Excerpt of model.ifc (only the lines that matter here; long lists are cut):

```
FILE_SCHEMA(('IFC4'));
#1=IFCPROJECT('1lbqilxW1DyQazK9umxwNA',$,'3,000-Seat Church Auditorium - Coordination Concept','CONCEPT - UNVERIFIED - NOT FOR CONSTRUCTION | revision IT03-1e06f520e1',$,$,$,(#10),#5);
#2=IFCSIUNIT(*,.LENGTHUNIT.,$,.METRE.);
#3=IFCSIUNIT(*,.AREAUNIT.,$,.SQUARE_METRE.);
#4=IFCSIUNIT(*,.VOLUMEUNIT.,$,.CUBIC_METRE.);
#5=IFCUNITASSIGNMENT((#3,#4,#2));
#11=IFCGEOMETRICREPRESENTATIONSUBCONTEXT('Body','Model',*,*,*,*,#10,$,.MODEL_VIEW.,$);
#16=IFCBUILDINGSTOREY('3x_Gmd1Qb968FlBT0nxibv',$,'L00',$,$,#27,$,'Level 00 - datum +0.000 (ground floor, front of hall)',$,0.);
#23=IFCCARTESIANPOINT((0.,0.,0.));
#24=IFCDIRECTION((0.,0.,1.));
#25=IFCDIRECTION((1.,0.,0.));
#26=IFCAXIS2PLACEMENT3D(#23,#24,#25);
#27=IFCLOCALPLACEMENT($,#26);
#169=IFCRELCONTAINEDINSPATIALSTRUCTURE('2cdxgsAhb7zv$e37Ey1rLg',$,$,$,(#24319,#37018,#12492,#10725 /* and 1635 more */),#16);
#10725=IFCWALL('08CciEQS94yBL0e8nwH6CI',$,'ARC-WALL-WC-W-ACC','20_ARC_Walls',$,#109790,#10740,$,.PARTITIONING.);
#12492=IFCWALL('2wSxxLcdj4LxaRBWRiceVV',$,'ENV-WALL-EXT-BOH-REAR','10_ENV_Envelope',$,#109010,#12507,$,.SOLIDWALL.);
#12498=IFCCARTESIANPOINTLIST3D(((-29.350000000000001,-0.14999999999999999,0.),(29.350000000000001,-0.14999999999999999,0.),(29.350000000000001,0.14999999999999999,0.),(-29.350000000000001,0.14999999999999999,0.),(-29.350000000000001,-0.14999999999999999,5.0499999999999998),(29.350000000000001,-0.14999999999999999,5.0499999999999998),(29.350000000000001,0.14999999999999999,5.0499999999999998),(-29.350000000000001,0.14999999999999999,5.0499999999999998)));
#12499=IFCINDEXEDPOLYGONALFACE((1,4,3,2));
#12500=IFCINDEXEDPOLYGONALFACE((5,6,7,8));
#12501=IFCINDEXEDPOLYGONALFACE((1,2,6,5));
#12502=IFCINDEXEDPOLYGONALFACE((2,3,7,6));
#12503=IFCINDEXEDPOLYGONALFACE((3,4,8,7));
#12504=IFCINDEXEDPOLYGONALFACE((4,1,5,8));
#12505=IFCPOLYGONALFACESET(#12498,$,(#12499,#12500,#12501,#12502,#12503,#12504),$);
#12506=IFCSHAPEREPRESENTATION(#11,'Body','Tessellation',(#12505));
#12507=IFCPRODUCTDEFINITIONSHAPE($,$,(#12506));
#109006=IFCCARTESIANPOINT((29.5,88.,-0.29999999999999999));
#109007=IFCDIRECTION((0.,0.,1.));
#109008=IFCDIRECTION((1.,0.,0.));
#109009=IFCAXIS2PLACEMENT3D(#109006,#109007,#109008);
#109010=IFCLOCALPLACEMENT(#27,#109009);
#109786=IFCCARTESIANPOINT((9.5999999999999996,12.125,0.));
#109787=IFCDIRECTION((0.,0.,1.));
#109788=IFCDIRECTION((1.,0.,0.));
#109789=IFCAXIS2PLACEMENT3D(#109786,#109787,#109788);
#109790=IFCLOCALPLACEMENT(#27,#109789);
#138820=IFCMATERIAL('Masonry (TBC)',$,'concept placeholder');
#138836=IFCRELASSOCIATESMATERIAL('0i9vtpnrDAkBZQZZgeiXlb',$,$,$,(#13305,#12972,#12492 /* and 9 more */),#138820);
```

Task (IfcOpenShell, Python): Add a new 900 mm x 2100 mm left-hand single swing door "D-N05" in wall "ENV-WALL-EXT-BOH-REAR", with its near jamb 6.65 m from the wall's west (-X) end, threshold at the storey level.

```python
import numpy as np
import ifcopenshell
import ifcopenshell.api.feature
import ifcopenshell.api.geometry
import ifcopenshell.api.root
import ifcopenshell.api.spatial
import ifcopenshell.geom
import ifcopenshell.util.element
import ifcopenshell.util.placement
import ifcopenshell.util.representation
import ifcopenshell.util.shape
import ifcopenshell.util.unit

model = ifcopenshell.open("model.ifc")
unit_scale = ifcopenshell.util.unit.calculate_unit_scale(model)
settings = ifcopenshell.geom.settings()


def volume(element):
    """Net volume in cubic metres, openings subtracted."""
    shape = ifcopenshell.geom.create_shape(settings, element)
    return ifcopenshell.util.shape.get_volume(shape.geometry)


wall = model.by_guid("2wSxxLcdj4LxaRBWRiceVV")
storey = ifcopenshell.util.element.get_container(wall, ifc_class="IfcBuildingStorey")
context = ifcopenshell.util.representation.get_context(model, "Model", "Body", "MODEL_VIEW")
before = volume(wall)

width, height, from_end, sill = 0.9, 2.1, 6.65, 0.0  # metres

# The wall runs along its own X axis, and the end named is its -X end.
wall_shape = ifcopenshell.geom.create_shape(settings, wall)
x, y, z = ifcopenshell.util.shape.get_vertices(wall_shape.geometry).T
start = x.min() + from_end
face, thickness = float(y.min()), float(y.max() - y.min())
wall_matrix = ifcopenshell.util.placement.get_local_placement(wall.ObjectPlacement)
level = ifcopenshell.util.placement.get_local_placement(storey.ObjectPlacement)[2, 3]


def in_wall(x, y):
    """Placement at x, y metres in the wall's axes, at sill height."""
    matrix = wall_matrix.copy()
    matrix[:, 3] = wall_matrix @ np.array([x / unit_scale, y / unit_scale, 0.0, 1.0])
    matrix[2, 3] = level + sill / unit_scale
    return matrix


# Opening: a box that overshoots both wall faces by 50 mm.
opening = ifcopenshell.api.root.create_entity(model, ifc_class="IfcOpeningElement", predefined_type="OPENING")
box = ifcopenshell.api.geometry.add_wall_representation(
    model, context=context, length=width, height=height, thickness=thickness + 0.1
)
ifcopenshell.api.geometry.assign_representation(model, product=opening, representation=box)
ifcopenshell.api.geometry.edit_object_placement(model, product=opening, matrix=in_wall(start, face - 0.05), is_si=False)
ifcopenshell.api.feature.add_feature(model, feature=opening, element=wall)

door = ifcopenshell.api.root.create_entity(model, ifc_class="IfcDoor", name="D-N05", predefined_type="DOOR")
door.OverallWidth, door.OverallHeight = width / unit_scale, height / unit_scale
door.OperationType = "SINGLE_SWING_LEFT"
body = ifcopenshell.api.geometry.add_door_representation(
    model,
    context=context,
    overall_width=door.OverallWidth,
    overall_height=door.OverallHeight,
    operation_type="SINGLE_SWING_LEFT",
    lining_properties={"LiningDepth": thickness / unit_scale, "ThresholdDepth": thickness / unit_scale},
)
ifcopenshell.api.geometry.assign_representation(model, product=door, representation=body)
ifcopenshell.api.spatial.assign_container(model, products=[door], relating_structure=storey)
ifcopenshell.api.feature.add_filling(model, opening=opening, element=door)

# The lining spans the wall, so the door starts at the wall face.
ifcopenshell.api.geometry.edit_object_placement(model, product=door, matrix=in_wall(start, face), is_si=False)

after = volume(wall)

print(f"wall volume {before:.3f} -> {after:.3f} m3")

model.write("model_updated.ifc")
```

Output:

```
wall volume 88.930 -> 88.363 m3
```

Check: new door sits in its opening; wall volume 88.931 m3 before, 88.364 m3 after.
